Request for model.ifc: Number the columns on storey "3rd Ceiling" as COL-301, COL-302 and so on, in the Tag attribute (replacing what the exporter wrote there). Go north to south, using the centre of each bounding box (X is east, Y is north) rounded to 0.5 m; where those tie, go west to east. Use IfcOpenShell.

First a look at what the model holds.

```python
import ifcopenshell
import ifcopenshell.util.element
import ifcopenshell.util.placement

model = ifcopenshell.open("model.ifc")
print(model.schema)
storey = next(s for s in model.by_type("IfcBuildingStorey") if s.Name == "3rd Ceiling")
columns = [e for e in ifcopenshell.util.element.get_decomposition(storey) if e.is_a("IfcColumn")]
for e in sorted(columns, key=lambda e: e.id()):
    origin = ifcopenshell.util.placement.get_local_placement(e.ObjectPlacement)[:3, 3]
    print(e.id(), e.Tag, e.Name, origin.round(2) + 0.0, sep=" | ")
```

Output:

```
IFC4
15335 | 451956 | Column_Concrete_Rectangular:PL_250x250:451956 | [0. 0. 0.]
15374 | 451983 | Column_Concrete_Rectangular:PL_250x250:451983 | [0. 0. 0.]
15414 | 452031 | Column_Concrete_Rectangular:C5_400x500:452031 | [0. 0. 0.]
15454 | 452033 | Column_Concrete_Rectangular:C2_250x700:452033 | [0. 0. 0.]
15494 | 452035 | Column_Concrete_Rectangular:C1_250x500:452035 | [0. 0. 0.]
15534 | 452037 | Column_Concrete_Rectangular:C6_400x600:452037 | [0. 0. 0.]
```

```python
import ifcopenshell
import ifcopenshell.geom
import ifcopenshell.util.element
import ifcopenshell.util.shape

model = ifcopenshell.open("model.ifc")
settings = ifcopenshell.geom.settings()
settings.set("use-world-coords", True)


def centre(element):
    shape = ifcopenshell.geom.create_shape(settings, element)
    return ifcopenshell.util.shape.get_bbox_centroid(shape.geometry)


storey = next(s for s in model.by_type("IfcBuildingStorey") if s.Name == "3rd Ceiling")
columns = [e for e in ifcopenshell.util.element.get_decomposition(storey) if e.is_a("IfcColumn")]

# Insertion points can sit at a corner or the storey origin, so sort by the geometry (in metres).
centres = {e: centre(e) for e in columns}
columns.sort(key=lambda e: (-round(centres[e][1] / 0.5), centres[e][0]))

for i, e in enumerate(columns, start=1):
    number = f"COL-3{i:02d}"
    e.Tag = number
    print(e.id(), number)

model.write("model_rev.ifc")
```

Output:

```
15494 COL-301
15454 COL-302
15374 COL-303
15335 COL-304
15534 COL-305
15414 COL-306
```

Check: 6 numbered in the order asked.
